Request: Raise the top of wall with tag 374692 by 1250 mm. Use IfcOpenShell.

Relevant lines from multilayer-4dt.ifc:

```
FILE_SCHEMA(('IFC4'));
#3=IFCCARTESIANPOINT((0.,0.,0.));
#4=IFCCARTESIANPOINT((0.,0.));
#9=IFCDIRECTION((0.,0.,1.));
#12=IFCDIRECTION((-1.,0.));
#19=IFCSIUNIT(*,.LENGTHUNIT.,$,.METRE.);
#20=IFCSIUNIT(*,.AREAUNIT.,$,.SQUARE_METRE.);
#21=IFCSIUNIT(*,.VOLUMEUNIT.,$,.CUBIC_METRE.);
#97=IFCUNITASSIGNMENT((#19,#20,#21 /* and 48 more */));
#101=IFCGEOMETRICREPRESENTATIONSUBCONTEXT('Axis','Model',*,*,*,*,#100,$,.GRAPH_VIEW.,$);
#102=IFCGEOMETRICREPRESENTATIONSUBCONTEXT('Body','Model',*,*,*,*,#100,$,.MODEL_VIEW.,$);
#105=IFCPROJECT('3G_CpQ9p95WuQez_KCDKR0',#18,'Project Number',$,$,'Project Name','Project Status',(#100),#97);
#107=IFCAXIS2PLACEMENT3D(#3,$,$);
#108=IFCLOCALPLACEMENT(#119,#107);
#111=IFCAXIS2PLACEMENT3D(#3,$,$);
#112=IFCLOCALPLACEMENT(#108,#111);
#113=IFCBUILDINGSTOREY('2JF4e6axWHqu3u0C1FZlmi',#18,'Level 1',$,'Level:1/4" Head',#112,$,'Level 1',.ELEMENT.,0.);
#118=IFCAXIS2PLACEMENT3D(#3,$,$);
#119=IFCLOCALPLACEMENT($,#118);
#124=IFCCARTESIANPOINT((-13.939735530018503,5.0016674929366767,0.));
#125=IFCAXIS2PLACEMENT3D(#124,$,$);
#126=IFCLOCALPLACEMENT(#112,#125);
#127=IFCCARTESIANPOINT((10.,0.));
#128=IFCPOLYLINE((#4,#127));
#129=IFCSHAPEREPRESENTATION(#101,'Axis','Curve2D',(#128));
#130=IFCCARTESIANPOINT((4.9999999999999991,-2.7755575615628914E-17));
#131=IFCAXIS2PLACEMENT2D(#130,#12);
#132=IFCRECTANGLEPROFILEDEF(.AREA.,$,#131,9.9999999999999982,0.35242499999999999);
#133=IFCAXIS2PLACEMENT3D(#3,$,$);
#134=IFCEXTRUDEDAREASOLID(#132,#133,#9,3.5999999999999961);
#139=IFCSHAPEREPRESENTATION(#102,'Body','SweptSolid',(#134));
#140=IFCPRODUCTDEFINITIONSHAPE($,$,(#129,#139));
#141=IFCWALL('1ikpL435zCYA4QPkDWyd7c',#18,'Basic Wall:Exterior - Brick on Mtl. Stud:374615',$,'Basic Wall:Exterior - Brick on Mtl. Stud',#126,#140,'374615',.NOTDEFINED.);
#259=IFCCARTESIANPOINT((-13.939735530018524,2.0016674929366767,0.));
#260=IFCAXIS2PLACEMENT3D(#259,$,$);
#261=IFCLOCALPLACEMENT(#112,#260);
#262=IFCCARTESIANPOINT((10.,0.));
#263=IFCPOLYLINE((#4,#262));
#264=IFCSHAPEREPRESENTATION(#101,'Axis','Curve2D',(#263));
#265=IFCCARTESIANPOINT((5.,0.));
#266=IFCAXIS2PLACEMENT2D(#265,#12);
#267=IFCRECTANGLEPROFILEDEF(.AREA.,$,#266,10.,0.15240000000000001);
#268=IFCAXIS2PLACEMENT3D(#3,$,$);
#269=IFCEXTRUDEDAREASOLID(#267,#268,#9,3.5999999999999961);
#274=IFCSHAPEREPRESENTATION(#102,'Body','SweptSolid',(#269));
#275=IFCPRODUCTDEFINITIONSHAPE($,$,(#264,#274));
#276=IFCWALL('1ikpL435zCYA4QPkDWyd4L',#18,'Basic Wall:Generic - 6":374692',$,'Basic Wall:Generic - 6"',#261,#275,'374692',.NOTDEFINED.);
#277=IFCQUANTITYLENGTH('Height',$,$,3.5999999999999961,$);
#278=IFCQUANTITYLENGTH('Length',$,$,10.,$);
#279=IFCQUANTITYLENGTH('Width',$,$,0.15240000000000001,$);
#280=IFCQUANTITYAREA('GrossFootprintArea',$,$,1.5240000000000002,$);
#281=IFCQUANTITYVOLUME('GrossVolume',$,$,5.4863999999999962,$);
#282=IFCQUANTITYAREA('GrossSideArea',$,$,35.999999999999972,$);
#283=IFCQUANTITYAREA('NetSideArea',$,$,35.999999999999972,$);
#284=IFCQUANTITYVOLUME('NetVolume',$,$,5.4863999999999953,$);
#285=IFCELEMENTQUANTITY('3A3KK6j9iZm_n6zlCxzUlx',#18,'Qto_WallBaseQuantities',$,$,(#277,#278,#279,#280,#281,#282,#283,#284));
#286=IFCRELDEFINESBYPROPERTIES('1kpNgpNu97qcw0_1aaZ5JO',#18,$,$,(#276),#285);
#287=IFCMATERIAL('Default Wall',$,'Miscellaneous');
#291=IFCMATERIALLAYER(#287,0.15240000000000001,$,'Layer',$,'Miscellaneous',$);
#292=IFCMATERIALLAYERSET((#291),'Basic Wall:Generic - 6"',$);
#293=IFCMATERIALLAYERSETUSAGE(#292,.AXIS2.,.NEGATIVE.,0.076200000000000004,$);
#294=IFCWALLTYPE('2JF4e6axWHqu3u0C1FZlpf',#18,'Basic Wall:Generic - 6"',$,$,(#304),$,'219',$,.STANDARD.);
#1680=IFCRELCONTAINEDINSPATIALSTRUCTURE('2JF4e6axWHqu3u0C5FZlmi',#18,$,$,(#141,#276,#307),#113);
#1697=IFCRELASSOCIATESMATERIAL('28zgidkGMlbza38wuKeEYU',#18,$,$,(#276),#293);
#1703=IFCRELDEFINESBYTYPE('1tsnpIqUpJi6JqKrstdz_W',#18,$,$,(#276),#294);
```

```python
import ifcopenshell
import ifcopenshell.api.pset
import ifcopenshell.geom
import ifcopenshell.util.element
import ifcopenshell.util.representation
import ifcopenshell.util.shape
import ifcopenshell.util.unit

model = ifcopenshell.open("multilayer-4dt.ifc")
unit_scale = ifcopenshell.util.unit.calculate_unit_scale(model)
area_scale = ifcopenshell.util.unit.calculate_unit_scale(model, "AREAUNIT")
volume_scale = ifcopenshell.util.unit.calculate_unit_scale(model, "VOLUMEUNIT")
settings = ifcopenshell.geom.settings()


def volume(element):
    """Net volume in cubic metres, openings subtracted."""
    shape = ifcopenshell.geom.create_shape(settings, element)
    return ifcopenshell.util.shape.get_volume(shape.geometry)


wall = model.by_guid("1ikpL435zCYA4QPkDWyd4L")
before = volume(wall)

body = ifcopenshell.util.representation.get_representation(wall, "Model", "Body")
solid = body.Items[0]
old_height = solid.Depth
solid.Depth += 1.25
after = volume(wall)
thickness = 0.1524  # wall thickness in metres

# Update the stored height, areas and volumes.
qto = model.by_id(ifcopenshell.util.element.get_pset(wall, "Qto_WallBaseQuantities", should_inherit=False)["id"])
ifcopenshell.api.pset.edit_qto(model, qto=qto, properties={
    "Height": solid.Depth,
    "GrossVolume": ifcopenshell.util.element.get_pset(wall, "Qto_WallBaseQuantities", "GrossVolume") * solid.Depth / old_height,
    "GrossSideArea": ifcopenshell.util.element.get_pset(wall, "Qto_WallBaseQuantities", "GrossSideArea") * solid.Depth / old_height,
    "NetSideArea": after / thickness / area_scale,
    "NetVolume": after / volume_scale,
})

print(f"height {old_height:g} -> {solid.Depth:g}, volume {before:.3f} -> {after:.3f} m3")

model.write("multilayer-4dt_v2.ifc")
```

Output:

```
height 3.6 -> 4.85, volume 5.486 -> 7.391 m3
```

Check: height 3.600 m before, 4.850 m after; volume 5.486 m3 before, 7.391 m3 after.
